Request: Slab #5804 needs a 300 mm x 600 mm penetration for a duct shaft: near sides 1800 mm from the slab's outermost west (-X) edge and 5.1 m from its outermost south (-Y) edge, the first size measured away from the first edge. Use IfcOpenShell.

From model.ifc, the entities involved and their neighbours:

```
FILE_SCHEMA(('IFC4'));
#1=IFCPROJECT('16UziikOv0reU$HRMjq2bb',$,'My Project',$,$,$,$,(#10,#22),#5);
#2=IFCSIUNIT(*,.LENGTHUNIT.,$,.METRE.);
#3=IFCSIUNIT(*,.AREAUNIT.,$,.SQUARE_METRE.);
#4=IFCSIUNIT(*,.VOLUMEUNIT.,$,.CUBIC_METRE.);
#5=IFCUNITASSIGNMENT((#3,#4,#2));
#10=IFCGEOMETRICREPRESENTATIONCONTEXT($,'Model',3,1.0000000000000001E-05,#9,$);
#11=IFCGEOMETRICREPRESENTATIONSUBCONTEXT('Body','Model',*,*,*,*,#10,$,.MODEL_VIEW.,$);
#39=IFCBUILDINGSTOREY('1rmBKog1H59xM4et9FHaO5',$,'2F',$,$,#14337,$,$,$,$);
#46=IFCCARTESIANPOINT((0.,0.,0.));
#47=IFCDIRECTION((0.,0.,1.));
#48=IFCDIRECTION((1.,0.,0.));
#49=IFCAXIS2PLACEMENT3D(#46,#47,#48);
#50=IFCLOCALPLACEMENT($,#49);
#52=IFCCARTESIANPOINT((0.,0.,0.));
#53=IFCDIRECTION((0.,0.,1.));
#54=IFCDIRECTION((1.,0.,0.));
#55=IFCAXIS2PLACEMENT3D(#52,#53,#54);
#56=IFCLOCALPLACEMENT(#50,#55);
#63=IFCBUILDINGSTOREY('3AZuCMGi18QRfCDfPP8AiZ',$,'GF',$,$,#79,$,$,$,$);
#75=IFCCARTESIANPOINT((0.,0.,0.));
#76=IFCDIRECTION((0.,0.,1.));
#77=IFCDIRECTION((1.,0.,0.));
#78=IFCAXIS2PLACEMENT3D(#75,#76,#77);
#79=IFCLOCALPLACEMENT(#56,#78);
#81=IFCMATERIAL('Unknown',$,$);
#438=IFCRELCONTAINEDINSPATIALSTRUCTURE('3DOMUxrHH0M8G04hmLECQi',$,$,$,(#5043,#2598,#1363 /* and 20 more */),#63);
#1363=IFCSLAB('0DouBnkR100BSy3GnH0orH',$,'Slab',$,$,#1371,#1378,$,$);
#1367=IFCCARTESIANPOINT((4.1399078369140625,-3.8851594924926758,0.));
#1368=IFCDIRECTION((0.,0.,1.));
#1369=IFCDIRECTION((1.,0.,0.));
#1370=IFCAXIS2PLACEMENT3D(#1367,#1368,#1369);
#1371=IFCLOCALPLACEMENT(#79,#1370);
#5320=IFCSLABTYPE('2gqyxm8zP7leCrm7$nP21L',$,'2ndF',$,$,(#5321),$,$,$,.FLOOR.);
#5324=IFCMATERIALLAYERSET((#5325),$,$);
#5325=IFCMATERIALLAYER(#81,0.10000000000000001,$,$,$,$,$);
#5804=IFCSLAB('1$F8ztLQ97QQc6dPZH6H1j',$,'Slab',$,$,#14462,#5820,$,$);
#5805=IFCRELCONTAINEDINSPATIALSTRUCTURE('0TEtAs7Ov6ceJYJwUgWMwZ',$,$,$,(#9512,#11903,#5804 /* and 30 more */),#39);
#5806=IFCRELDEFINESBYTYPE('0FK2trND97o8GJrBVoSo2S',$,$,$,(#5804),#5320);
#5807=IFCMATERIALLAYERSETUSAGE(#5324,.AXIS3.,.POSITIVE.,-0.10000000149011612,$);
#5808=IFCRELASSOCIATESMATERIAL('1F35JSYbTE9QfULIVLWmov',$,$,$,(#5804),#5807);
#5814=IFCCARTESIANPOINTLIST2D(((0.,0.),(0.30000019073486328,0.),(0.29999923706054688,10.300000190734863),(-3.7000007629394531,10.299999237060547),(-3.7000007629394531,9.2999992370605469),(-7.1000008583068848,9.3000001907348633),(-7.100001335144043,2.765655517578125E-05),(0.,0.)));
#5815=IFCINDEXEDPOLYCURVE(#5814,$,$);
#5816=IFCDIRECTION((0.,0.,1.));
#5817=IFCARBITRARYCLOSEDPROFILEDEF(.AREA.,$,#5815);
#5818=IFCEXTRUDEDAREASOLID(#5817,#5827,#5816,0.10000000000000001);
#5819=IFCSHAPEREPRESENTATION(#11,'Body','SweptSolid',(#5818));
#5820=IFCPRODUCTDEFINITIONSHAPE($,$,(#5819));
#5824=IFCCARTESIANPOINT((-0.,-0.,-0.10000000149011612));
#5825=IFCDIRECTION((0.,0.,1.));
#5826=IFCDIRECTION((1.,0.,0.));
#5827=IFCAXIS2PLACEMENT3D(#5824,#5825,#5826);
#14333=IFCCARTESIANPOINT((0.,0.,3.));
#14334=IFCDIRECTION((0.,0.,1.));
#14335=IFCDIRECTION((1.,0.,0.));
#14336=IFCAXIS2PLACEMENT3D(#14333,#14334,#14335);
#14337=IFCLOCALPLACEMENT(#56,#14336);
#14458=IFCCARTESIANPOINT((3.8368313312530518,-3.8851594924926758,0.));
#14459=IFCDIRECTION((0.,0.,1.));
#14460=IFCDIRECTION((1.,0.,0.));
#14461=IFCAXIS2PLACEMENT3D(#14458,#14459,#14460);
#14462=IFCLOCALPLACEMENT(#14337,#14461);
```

```python
import numpy as np
import ifcopenshell
import ifcopenshell.api.feature
import ifcopenshell.api.geometry
import ifcopenshell.api.root
import ifcopenshell.geom
import ifcopenshell.util.placement
import ifcopenshell.util.representation
import ifcopenshell.util.shape
import ifcopenshell.util.unit

model = ifcopenshell.open("model.ifc")
unit_scale = ifcopenshell.util.unit.calculate_unit_scale(model)
settings = ifcopenshell.geom.settings()


def volume(element):
    """Net volume in cubic metres, openings subtracted."""
    shape = ifcopenshell.geom.create_shape(settings, element)
    return ifcopenshell.util.shape.get_volume(shape.geometry)


slab = model.by_guid("1$F8ztLQ97QQc6dPZH6H1j")
before = volume(slab)

# Extent in the slab's own axes, in metres. The edges named are its -X and -Y sides.
slab_shape = ifcopenshell.geom.create_shape(settings, slab)
vertices = ifcopenshell.util.shape.get_vertices(slab_shape.geometry)
x_min, y_min, bottom = vertices.min(axis=0)
top = vertices[:, 2].max()

opening = ifcopenshell.api.root.create_entity(model, ifc_class="IfcOpeningElement", name="Duct shaft opening", predefined_type="OPENING")
context = ifcopenshell.util.representation.get_context(model, "Model", "Body", "MODEL_VIEW")
width, depth = 0.3, 0.6
outline = [(0.0, 0.0), (width, 0.0), (width, depth), (0.0, depth), (0.0, 0.0)]
# Overshoot both faces by 50 mm so the cut is clean.
shape = ifcopenshell.api.geometry.add_slab_representation(
    model, context=context, depth=top - bottom + 0.1, polyline=outline
)
ifcopenshell.api.geometry.assign_representation(model, product=opening, representation=shape)

matrix = ifcopenshell.util.placement.get_local_placement(slab.ObjectPlacement)
matrix[:, 3] = matrix @ np.append(np.array([x_min + 1.8, y_min + 5.1, bottom - 0.05]) / unit_scale, 1.0)
ifcopenshell.api.geometry.edit_object_placement(model, product=opening, matrix=matrix, is_si=False)
ifcopenshell.api.feature.add_feature(model, feature=opening, element=slab)

after = volume(slab)

print(f"slab volume {before:.3f} -> {after:.3f} m3")

model.write("model_rev.ifc")
```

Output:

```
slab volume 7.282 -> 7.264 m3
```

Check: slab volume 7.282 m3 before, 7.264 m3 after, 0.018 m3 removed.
